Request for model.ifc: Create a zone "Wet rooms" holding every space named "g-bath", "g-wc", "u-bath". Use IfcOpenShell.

First a look at what the model holds.

```python
import ifcopenshell

model = ifcopenshell.open("model.ifc")
print(model.schema)
seen = {}
for space in model.by_type("IfcSpace"):
    seen[space.LongName] = seen.get(space.LongName, 0) + 1
for name, count in sorted(seen.items(), key=str):
    print(count, "x", name)
print("zones:", [z.Name for z in model.by_type("IfcZone")][:20])
```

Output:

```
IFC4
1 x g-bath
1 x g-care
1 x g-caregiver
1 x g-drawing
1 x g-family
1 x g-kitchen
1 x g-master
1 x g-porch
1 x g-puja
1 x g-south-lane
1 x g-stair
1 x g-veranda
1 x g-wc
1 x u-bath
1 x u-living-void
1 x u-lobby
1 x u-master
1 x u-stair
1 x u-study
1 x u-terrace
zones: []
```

```python
import ifcopenshell
import ifcopenshell.api.group
import ifcopenshell.api.root

model = ifcopenshell.open("model.ifc")

names = {"g-bath", "g-wc", "u-bath"}
spaces = [s for s in model.by_type("IfcSpace") if s.LongName in names]

zone = ifcopenshell.api.root.create_entity(model, ifc_class="IfcZone", name="Wet rooms")
ifcopenshell.api.group.assign_group(model, products=spaces, group=zone)
print(len(spaces), "spaces in", zone.Name)

model.write("model_v2.ifc")
```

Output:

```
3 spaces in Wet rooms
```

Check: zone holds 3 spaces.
